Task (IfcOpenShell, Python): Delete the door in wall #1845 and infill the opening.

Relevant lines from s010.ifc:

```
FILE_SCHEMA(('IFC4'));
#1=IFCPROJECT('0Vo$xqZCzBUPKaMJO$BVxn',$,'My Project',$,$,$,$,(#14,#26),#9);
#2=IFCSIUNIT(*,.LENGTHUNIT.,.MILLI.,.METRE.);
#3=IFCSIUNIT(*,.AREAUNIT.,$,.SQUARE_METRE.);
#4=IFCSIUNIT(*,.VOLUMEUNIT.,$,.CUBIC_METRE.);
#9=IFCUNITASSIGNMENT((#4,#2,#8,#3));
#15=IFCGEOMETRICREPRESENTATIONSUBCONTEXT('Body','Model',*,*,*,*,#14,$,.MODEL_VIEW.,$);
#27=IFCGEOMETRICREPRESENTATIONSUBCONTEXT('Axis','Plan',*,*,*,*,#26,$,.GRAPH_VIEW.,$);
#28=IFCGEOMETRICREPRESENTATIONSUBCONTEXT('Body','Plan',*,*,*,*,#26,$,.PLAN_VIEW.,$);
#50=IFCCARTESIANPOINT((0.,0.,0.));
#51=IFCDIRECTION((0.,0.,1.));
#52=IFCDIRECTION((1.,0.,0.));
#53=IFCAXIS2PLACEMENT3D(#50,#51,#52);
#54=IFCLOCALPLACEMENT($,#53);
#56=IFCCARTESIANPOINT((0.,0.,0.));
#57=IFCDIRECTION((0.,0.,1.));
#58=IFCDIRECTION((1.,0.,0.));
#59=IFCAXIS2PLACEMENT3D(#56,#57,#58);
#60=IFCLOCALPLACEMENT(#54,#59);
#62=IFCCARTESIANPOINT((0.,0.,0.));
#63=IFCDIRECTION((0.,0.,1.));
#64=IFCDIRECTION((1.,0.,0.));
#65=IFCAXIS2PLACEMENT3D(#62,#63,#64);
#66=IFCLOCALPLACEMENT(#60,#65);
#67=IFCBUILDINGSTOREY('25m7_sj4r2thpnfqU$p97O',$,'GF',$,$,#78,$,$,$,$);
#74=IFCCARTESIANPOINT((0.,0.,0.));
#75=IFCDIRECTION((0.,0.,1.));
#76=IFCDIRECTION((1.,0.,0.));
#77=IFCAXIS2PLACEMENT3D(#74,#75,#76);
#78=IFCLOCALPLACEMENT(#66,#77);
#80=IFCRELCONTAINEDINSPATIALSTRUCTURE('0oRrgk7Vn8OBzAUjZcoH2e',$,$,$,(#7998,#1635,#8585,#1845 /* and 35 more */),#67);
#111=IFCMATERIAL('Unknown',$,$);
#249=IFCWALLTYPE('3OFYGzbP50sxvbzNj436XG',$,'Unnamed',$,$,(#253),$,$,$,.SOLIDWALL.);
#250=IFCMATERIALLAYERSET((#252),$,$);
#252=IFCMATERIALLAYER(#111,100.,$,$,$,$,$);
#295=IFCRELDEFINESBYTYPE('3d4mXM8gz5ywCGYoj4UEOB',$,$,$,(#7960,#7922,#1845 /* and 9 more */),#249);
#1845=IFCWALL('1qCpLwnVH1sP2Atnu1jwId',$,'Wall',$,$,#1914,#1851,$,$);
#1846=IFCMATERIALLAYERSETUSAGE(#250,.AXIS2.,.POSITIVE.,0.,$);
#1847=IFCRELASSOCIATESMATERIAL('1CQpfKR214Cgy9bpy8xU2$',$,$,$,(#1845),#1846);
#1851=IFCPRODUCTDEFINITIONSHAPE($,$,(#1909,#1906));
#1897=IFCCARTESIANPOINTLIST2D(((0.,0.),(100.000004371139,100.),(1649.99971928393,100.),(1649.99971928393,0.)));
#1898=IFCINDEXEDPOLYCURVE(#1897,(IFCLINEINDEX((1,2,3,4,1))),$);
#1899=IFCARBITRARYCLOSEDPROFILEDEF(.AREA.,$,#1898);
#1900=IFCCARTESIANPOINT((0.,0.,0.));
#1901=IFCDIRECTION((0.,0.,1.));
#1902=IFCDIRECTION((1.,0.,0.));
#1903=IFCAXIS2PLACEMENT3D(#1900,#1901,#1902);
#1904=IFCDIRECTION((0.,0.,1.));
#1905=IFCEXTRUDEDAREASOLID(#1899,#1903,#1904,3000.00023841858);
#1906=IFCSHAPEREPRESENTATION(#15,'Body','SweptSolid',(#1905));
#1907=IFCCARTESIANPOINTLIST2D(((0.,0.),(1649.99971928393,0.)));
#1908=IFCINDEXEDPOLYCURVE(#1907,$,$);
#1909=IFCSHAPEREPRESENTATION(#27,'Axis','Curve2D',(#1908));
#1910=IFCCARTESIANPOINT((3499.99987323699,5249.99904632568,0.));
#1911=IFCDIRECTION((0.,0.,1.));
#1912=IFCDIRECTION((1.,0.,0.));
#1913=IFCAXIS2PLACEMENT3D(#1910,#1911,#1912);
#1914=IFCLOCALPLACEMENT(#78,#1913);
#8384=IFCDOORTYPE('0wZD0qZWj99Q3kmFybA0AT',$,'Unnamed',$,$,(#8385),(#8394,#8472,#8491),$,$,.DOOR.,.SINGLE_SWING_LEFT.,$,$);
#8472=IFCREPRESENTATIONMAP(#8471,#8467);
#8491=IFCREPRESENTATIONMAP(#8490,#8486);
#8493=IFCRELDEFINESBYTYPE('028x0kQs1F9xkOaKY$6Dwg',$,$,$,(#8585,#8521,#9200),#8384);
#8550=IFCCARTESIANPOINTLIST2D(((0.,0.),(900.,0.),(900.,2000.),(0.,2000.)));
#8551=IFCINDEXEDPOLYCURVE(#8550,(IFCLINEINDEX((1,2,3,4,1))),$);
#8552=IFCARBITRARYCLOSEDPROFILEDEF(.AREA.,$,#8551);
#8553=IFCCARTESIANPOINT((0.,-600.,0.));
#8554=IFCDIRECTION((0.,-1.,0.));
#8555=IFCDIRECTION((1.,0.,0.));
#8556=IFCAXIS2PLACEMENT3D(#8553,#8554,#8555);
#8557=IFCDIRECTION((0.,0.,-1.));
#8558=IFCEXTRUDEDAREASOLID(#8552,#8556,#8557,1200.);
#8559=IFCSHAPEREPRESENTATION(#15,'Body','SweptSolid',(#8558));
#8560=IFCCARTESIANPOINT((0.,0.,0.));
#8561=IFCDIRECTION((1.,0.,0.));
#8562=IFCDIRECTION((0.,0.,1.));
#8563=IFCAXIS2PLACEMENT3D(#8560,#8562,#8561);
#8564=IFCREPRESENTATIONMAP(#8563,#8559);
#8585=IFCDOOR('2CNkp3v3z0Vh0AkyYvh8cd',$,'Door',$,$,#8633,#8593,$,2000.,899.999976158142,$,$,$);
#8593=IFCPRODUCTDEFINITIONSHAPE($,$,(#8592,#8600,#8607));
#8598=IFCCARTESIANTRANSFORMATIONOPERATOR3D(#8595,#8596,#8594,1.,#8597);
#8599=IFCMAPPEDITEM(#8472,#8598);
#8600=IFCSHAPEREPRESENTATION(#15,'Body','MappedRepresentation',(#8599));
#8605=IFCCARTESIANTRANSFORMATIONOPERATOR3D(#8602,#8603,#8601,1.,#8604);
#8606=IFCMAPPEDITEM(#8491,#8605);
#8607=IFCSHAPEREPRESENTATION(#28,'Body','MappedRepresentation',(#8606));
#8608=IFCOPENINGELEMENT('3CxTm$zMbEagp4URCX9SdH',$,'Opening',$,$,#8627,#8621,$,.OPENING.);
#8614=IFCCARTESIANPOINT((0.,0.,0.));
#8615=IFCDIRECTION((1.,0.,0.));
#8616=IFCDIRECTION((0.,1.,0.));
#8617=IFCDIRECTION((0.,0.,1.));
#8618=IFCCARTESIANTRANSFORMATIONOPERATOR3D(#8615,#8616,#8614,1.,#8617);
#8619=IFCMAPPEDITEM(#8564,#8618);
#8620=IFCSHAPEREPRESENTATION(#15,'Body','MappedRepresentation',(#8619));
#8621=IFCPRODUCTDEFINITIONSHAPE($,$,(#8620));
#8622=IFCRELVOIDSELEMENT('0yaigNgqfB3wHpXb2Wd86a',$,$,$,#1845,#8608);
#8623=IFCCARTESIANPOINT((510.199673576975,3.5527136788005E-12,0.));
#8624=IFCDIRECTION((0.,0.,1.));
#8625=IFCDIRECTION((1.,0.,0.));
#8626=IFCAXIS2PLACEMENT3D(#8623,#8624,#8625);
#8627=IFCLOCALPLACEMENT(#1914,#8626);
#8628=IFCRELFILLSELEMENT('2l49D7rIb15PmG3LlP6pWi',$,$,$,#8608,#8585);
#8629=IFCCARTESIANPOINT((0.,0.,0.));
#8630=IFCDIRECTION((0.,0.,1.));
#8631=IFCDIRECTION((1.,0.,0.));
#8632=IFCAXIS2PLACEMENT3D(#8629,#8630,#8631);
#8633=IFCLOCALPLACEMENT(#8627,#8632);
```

```python
import ifcopenshell
import ifcopenshell.api.feature
import ifcopenshell.api.root
import ifcopenshell.geom
import ifcopenshell.util.shape

model = ifcopenshell.open("s010.ifc")
settings = ifcopenshell.geom.settings()


def volume(element):
    """Net volume in cubic metres, openings subtracted."""
    shape = ifcopenshell.geom.create_shape(settings, element)
    return ifcopenshell.util.shape.get_volume(shape.geometry)


door = model.by_guid("2CNkp3v3z0Vh0AkyYvh8cd")
opening = door.FillsVoids[0].RelatingOpeningElement
wall = opening.VoidsElements[0].RelatingBuildingElement
before = volume(wall)

ifcopenshell.api.root.remove_product(model, product=door)
ifcopenshell.api.feature.remove_feature(model, feature=opening)

after = volume(wall)

print(f"wall volume {before:.3f} -> {after:.3f} m3")

model.write("s010_v2.ifc")
```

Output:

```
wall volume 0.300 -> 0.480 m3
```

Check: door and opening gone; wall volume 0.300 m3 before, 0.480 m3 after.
